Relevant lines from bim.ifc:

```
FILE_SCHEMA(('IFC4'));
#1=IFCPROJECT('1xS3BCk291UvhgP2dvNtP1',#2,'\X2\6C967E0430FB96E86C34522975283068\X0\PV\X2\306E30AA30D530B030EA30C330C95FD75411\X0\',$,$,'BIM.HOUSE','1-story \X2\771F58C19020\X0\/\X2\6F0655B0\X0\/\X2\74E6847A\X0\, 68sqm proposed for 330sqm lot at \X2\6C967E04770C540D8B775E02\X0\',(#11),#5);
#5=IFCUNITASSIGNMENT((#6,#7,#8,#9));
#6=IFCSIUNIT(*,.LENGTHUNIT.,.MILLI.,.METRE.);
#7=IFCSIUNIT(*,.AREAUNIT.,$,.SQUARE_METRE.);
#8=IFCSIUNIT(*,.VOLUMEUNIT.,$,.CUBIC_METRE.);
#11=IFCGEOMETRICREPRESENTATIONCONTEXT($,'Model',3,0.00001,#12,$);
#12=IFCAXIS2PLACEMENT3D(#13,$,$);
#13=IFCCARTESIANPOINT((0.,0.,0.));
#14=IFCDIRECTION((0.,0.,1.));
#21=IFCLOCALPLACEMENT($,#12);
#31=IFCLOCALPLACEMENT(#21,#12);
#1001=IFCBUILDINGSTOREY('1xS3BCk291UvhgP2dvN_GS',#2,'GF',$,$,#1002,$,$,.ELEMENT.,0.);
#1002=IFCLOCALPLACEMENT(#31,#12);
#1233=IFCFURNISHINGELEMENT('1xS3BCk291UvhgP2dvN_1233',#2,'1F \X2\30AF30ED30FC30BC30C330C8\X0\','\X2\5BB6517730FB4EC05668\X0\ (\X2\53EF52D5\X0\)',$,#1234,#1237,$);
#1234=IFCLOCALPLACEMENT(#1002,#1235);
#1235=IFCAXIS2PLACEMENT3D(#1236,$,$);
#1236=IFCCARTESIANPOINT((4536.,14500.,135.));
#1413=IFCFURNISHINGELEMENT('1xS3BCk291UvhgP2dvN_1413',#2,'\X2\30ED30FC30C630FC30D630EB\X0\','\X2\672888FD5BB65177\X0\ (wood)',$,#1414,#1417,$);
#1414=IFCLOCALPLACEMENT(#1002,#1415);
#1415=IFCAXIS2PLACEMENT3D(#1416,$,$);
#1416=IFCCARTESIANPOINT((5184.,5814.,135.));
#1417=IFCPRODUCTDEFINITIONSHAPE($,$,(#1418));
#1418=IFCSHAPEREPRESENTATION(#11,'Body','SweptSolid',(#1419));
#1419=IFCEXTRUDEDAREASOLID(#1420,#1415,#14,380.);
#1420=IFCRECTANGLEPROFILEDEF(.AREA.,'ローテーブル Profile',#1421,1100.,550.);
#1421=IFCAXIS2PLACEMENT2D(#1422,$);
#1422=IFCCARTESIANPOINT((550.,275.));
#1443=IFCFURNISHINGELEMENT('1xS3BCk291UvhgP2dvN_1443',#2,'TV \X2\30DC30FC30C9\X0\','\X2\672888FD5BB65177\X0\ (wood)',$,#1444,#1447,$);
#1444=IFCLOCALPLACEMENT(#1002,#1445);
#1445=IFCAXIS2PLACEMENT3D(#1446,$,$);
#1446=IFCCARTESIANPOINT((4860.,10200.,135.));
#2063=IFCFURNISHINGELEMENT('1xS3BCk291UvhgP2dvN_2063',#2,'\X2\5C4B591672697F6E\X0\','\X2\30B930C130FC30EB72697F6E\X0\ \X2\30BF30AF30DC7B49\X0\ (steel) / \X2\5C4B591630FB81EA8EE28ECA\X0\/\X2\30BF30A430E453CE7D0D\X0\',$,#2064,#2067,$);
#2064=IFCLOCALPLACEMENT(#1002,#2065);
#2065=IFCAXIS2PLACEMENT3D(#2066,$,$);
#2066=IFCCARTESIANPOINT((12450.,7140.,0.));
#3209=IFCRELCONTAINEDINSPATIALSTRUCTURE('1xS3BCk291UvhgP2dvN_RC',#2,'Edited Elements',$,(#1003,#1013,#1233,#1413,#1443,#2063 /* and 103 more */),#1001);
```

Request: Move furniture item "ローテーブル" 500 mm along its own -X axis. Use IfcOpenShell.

```python
import ifcopenshell
import ifcopenshell.api.geometry
import ifcopenshell.util.placement

model = ifcopenshell.open("bim.ifc")

item = model.by_guid("1xS3BCk291UvhgP2dvN_1413")
matrix = ifcopenshell.util.placement.get_local_placement(item.ObjectPlacement)
matrix[:3, 3] -= matrix[:3, 0] * 500.0
ifcopenshell.api.geometry.edit_object_placement(model, product=item, matrix=matrix, is_si=False)

print(ifcopenshell.util.placement.get_local_placement(item.ObjectPlacement).round(3) + 0.0)

model.write("bim-out.ifc")
```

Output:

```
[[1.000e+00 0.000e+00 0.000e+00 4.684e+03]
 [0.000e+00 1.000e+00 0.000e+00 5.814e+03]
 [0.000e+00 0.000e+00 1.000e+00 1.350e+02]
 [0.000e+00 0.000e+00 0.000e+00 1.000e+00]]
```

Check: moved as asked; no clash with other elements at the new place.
